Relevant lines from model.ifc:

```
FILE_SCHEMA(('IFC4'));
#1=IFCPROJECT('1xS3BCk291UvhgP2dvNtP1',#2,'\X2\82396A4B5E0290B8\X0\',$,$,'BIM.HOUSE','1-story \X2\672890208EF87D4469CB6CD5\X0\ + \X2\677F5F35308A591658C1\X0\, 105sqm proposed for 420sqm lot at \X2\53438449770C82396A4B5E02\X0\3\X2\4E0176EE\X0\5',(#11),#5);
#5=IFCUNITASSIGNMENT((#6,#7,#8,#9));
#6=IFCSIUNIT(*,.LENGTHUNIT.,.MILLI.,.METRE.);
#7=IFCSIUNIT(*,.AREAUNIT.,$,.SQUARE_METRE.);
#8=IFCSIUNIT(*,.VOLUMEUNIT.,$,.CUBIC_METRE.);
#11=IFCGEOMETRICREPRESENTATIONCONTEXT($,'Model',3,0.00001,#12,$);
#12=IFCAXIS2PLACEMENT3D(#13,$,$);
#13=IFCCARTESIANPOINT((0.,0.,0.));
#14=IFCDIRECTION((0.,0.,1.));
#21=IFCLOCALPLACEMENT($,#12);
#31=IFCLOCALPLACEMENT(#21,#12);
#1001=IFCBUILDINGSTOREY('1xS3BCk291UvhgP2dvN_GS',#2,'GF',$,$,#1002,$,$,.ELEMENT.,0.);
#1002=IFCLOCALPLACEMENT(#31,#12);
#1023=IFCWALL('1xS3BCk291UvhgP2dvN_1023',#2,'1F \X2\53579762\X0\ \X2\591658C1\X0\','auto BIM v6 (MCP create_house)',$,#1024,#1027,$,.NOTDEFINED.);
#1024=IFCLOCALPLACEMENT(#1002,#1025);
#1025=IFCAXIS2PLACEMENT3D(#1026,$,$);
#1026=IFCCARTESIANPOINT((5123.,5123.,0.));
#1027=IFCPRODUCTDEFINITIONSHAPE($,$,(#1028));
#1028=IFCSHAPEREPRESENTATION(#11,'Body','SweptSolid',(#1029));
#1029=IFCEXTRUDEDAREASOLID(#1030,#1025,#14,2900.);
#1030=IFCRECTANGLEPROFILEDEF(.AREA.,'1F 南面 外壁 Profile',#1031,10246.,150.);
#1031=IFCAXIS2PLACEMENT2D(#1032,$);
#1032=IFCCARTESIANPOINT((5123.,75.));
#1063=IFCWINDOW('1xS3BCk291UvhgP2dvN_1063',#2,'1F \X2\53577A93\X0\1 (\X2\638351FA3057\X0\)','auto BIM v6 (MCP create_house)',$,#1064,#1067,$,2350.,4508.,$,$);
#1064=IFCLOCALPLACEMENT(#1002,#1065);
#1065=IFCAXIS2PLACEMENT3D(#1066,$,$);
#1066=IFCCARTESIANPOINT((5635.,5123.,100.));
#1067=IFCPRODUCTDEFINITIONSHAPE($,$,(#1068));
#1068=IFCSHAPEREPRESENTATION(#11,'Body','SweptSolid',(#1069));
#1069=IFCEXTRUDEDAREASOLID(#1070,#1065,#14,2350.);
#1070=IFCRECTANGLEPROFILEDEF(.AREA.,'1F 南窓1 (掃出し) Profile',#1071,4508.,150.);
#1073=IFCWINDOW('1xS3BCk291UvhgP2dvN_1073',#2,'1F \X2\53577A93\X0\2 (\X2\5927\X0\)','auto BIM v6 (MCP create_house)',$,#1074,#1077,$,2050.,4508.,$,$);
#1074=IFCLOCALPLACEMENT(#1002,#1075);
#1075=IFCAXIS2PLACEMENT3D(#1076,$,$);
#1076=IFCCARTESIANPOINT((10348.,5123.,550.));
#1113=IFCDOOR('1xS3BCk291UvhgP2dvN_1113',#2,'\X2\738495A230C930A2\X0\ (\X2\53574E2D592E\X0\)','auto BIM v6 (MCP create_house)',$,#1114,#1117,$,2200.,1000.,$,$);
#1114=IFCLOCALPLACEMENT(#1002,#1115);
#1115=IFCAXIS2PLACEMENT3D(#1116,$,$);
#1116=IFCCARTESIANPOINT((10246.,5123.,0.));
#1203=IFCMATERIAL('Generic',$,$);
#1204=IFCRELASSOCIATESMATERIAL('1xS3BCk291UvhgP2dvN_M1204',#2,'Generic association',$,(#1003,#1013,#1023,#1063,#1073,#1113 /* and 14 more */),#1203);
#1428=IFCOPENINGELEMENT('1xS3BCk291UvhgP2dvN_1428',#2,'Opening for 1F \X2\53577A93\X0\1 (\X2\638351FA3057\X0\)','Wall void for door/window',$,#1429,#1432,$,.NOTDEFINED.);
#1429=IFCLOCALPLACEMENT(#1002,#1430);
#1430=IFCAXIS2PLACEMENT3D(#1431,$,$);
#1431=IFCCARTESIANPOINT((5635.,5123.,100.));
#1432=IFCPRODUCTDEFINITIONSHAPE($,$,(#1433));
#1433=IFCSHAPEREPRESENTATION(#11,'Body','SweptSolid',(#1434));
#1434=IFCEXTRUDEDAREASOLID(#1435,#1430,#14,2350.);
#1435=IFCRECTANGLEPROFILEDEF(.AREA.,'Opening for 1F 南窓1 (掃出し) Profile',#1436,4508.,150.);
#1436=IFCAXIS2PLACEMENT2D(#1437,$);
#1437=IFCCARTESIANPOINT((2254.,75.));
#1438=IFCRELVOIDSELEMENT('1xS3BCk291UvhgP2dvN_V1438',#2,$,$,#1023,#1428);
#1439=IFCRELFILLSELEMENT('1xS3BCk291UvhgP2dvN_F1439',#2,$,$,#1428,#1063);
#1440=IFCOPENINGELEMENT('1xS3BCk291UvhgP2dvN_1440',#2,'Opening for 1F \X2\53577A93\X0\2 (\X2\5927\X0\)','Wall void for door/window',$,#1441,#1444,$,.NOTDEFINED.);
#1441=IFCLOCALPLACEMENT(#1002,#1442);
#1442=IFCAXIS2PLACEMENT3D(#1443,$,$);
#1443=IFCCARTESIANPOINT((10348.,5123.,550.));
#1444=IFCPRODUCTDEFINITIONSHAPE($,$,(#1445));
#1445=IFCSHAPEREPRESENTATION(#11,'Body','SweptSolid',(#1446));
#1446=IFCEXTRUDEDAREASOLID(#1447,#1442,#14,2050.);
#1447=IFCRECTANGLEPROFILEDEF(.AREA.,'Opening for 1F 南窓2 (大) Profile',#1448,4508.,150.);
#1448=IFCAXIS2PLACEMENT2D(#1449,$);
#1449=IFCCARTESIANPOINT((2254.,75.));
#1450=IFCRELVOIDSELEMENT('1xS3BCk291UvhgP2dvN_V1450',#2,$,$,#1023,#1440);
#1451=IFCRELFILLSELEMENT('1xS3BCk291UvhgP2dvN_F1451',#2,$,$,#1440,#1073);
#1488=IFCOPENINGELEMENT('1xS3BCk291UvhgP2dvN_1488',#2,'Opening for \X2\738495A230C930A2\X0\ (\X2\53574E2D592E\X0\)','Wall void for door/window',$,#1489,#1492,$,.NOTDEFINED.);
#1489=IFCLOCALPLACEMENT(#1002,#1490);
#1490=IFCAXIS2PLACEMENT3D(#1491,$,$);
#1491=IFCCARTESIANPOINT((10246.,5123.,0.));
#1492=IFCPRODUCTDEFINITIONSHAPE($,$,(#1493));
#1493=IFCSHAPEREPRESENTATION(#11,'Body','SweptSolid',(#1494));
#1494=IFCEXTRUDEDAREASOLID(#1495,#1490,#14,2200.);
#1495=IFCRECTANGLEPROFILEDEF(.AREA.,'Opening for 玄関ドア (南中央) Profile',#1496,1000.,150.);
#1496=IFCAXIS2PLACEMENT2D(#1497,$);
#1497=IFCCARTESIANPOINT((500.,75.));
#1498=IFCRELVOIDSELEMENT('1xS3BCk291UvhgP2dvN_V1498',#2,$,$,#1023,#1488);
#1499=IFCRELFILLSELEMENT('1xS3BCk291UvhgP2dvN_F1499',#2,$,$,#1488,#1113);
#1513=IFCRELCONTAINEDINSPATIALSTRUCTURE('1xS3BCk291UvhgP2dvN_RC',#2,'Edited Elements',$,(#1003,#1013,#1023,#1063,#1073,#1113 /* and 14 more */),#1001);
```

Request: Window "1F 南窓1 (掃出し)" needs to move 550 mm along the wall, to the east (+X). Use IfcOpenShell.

```python
import ifcopenshell
import ifcopenshell.api.geometry
import ifcopenshell.util.placement
import ifcopenshell.util.unit

model = ifcopenshell.open("model.ifc")
unit_scale = ifcopenshell.util.unit.calculate_unit_scale(model)

window = model.by_guid("1xS3BCk291UvhgP2dvN_1063")
opening = window.FillsVoids[0].RelatingOpeningElement
wall = opening.VoidsElements[0].RelatingBuildingElement

wall_matrix = ifcopenshell.util.placement.get_local_placement(wall.ObjectPlacement)
shift = wall_matrix[:3, 0] * 0.55 / unit_scale
before = ifcopenshell.util.placement.get_local_placement(window.ObjectPlacement)[:3, 3].copy()

# The window is not placed relative to its opening, so move both.
for product in (opening, window):
    matrix = ifcopenshell.util.placement.get_local_placement(product.ObjectPlacement)
    matrix[:3, 3] += shift
    ifcopenshell.api.geometry.edit_object_placement(model, product=product, matrix=matrix, is_si=False)

after = ifcopenshell.util.placement.get_local_placement(window.ObjectPlacement)[:3, 3]
print("window moved by", (after - before).round(3) + 0.0)

model.write("model_rev.ifc")
```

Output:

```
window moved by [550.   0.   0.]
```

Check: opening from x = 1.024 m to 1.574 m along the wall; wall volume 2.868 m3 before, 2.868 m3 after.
